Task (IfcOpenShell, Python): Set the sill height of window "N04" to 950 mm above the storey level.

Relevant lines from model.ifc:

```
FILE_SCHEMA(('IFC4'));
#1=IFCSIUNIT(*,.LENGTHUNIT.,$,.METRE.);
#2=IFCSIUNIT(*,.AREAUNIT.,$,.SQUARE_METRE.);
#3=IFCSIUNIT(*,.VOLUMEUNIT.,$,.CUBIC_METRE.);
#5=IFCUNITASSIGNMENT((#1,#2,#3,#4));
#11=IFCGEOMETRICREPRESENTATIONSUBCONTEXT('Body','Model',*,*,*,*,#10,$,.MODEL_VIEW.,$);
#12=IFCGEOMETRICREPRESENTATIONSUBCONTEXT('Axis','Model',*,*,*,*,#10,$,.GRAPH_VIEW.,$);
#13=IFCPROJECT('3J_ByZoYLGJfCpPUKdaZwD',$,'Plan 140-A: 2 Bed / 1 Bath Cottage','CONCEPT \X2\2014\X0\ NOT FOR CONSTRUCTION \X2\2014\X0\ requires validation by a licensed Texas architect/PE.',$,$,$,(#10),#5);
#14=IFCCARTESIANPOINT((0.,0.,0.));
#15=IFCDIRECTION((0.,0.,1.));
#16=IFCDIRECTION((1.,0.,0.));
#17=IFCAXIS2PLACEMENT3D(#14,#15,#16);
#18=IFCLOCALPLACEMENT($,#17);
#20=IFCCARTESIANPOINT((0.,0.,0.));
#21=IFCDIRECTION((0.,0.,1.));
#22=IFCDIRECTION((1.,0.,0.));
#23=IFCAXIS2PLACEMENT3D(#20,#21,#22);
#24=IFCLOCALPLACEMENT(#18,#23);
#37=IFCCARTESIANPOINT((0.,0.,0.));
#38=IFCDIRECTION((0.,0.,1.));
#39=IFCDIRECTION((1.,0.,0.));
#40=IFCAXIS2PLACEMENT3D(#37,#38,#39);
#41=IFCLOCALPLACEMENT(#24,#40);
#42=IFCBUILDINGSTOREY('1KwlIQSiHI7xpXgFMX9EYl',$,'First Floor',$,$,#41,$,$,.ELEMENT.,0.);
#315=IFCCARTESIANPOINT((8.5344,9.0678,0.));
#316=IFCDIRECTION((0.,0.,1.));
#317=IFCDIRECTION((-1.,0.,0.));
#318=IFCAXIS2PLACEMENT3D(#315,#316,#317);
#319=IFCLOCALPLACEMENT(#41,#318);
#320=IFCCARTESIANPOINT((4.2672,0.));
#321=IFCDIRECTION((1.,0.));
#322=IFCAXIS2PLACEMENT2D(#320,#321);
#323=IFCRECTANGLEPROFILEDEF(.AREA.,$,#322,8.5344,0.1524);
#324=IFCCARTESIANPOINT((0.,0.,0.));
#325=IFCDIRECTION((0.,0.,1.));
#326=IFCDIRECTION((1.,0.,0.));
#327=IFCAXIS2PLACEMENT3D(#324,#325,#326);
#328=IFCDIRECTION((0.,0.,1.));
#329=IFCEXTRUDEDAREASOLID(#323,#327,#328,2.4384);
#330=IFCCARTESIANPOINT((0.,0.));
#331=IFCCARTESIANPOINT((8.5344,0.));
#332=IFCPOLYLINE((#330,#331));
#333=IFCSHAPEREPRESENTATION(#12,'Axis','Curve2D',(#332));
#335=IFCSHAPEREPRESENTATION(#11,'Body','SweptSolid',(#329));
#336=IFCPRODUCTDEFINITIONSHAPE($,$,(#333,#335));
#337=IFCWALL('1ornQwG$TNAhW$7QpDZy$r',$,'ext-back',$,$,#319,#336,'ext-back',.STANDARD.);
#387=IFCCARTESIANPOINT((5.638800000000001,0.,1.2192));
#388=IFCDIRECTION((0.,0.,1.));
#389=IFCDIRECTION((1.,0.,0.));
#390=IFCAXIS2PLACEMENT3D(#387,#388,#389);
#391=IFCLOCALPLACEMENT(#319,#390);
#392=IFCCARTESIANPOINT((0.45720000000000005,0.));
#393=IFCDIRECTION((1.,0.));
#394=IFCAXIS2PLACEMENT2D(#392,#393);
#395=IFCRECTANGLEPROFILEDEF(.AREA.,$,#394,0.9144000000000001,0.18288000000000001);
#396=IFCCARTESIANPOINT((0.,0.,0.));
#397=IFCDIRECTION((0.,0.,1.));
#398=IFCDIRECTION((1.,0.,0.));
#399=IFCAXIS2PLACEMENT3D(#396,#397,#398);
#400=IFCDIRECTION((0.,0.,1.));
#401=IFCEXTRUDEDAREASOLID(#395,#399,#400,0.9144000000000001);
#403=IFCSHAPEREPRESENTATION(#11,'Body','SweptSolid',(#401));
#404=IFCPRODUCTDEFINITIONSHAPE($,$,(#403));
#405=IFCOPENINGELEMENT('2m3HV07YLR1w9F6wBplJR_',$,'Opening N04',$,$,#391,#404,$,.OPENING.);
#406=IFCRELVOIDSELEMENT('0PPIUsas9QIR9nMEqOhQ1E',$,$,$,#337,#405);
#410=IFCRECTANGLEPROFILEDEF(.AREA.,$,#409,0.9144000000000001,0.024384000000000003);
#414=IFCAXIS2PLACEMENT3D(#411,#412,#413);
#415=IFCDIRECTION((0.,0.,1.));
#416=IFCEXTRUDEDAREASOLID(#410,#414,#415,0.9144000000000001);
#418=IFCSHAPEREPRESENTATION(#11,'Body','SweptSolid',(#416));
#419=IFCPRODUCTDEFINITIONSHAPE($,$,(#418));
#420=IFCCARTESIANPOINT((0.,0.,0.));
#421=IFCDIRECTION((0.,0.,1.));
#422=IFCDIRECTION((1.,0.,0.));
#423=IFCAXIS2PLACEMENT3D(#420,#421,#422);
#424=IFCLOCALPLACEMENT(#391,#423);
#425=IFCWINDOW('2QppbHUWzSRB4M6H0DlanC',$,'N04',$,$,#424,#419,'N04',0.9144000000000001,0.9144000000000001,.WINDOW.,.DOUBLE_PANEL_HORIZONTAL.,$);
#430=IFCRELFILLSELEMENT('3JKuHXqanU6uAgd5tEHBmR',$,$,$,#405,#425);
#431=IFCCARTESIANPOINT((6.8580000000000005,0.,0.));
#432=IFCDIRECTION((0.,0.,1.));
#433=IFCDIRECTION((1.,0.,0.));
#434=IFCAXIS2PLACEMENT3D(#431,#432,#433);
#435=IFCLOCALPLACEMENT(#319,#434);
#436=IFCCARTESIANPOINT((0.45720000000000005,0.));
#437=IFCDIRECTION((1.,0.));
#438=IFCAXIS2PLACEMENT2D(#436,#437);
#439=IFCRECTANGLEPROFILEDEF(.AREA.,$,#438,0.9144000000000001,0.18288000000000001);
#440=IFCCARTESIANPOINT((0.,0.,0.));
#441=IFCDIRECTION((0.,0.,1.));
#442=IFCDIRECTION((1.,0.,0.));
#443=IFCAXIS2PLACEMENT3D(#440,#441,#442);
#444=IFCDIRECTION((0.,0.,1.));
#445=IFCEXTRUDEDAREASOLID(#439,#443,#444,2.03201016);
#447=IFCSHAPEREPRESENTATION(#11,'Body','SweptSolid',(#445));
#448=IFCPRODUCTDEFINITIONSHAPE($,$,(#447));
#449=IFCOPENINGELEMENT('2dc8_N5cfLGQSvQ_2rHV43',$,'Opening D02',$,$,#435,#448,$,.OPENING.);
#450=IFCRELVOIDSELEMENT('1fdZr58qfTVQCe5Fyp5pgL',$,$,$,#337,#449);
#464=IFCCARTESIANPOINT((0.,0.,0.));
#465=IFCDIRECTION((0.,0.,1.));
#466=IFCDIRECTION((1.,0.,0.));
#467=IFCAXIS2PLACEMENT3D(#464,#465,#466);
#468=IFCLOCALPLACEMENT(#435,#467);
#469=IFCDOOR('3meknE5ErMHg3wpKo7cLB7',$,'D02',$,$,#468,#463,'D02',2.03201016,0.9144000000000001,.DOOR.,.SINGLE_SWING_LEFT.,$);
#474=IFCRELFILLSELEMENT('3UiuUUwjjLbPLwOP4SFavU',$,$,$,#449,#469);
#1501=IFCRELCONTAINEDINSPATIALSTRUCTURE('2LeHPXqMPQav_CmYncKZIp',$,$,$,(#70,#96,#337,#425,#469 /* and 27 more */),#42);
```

```python
import numpy as np
import ifcopenshell
import ifcopenshell.api.geometry
import ifcopenshell.geom
import ifcopenshell.util.element
import ifcopenshell.util.placement
import ifcopenshell.util.shape
import ifcopenshell.util.unit

model = ifcopenshell.open("model.ifc")
unit_scale = ifcopenshell.util.unit.calculate_unit_scale(model)

window = model.by_guid("2QppbHUWzSRB4M6H0DlanC")
opening = window.FillsVoids[0].RelatingOpeningElement
storey = ifcopenshell.util.element.get_container(window, ifc_class="IfcBuildingStorey")
level = ifcopenshell.util.placement.get_local_placement(storey.ObjectPlacement)[2, 3]

# The opening's origin need not be at the sill, so measure its lowest point.
shape = ifcopenshell.geom.create_shape(ifcopenshell.geom.settings(), opening)
bottom = ifcopenshell.util.shape.get_shape_bottom_elevation(shape, shape.geometry) / unit_scale
dz = level + 0.95 - bottom

shift = np.array([0.0, 0.0, dz])
# The window is placed relative to its opening, so it follows when the opening moves.
matrix = ifcopenshell.util.placement.get_local_placement(opening.ObjectPlacement)
matrix[:3, 3] += shift
ifcopenshell.api.geometry.edit_object_placement(
    model, product=opening, matrix=matrix, is_si=False, should_transform_children=True
)

print(f"moved by {dz * unit_scale:+.3f} m")

model.write("model_edited.ifc")
```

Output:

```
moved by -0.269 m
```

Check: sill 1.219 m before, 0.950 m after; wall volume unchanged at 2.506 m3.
